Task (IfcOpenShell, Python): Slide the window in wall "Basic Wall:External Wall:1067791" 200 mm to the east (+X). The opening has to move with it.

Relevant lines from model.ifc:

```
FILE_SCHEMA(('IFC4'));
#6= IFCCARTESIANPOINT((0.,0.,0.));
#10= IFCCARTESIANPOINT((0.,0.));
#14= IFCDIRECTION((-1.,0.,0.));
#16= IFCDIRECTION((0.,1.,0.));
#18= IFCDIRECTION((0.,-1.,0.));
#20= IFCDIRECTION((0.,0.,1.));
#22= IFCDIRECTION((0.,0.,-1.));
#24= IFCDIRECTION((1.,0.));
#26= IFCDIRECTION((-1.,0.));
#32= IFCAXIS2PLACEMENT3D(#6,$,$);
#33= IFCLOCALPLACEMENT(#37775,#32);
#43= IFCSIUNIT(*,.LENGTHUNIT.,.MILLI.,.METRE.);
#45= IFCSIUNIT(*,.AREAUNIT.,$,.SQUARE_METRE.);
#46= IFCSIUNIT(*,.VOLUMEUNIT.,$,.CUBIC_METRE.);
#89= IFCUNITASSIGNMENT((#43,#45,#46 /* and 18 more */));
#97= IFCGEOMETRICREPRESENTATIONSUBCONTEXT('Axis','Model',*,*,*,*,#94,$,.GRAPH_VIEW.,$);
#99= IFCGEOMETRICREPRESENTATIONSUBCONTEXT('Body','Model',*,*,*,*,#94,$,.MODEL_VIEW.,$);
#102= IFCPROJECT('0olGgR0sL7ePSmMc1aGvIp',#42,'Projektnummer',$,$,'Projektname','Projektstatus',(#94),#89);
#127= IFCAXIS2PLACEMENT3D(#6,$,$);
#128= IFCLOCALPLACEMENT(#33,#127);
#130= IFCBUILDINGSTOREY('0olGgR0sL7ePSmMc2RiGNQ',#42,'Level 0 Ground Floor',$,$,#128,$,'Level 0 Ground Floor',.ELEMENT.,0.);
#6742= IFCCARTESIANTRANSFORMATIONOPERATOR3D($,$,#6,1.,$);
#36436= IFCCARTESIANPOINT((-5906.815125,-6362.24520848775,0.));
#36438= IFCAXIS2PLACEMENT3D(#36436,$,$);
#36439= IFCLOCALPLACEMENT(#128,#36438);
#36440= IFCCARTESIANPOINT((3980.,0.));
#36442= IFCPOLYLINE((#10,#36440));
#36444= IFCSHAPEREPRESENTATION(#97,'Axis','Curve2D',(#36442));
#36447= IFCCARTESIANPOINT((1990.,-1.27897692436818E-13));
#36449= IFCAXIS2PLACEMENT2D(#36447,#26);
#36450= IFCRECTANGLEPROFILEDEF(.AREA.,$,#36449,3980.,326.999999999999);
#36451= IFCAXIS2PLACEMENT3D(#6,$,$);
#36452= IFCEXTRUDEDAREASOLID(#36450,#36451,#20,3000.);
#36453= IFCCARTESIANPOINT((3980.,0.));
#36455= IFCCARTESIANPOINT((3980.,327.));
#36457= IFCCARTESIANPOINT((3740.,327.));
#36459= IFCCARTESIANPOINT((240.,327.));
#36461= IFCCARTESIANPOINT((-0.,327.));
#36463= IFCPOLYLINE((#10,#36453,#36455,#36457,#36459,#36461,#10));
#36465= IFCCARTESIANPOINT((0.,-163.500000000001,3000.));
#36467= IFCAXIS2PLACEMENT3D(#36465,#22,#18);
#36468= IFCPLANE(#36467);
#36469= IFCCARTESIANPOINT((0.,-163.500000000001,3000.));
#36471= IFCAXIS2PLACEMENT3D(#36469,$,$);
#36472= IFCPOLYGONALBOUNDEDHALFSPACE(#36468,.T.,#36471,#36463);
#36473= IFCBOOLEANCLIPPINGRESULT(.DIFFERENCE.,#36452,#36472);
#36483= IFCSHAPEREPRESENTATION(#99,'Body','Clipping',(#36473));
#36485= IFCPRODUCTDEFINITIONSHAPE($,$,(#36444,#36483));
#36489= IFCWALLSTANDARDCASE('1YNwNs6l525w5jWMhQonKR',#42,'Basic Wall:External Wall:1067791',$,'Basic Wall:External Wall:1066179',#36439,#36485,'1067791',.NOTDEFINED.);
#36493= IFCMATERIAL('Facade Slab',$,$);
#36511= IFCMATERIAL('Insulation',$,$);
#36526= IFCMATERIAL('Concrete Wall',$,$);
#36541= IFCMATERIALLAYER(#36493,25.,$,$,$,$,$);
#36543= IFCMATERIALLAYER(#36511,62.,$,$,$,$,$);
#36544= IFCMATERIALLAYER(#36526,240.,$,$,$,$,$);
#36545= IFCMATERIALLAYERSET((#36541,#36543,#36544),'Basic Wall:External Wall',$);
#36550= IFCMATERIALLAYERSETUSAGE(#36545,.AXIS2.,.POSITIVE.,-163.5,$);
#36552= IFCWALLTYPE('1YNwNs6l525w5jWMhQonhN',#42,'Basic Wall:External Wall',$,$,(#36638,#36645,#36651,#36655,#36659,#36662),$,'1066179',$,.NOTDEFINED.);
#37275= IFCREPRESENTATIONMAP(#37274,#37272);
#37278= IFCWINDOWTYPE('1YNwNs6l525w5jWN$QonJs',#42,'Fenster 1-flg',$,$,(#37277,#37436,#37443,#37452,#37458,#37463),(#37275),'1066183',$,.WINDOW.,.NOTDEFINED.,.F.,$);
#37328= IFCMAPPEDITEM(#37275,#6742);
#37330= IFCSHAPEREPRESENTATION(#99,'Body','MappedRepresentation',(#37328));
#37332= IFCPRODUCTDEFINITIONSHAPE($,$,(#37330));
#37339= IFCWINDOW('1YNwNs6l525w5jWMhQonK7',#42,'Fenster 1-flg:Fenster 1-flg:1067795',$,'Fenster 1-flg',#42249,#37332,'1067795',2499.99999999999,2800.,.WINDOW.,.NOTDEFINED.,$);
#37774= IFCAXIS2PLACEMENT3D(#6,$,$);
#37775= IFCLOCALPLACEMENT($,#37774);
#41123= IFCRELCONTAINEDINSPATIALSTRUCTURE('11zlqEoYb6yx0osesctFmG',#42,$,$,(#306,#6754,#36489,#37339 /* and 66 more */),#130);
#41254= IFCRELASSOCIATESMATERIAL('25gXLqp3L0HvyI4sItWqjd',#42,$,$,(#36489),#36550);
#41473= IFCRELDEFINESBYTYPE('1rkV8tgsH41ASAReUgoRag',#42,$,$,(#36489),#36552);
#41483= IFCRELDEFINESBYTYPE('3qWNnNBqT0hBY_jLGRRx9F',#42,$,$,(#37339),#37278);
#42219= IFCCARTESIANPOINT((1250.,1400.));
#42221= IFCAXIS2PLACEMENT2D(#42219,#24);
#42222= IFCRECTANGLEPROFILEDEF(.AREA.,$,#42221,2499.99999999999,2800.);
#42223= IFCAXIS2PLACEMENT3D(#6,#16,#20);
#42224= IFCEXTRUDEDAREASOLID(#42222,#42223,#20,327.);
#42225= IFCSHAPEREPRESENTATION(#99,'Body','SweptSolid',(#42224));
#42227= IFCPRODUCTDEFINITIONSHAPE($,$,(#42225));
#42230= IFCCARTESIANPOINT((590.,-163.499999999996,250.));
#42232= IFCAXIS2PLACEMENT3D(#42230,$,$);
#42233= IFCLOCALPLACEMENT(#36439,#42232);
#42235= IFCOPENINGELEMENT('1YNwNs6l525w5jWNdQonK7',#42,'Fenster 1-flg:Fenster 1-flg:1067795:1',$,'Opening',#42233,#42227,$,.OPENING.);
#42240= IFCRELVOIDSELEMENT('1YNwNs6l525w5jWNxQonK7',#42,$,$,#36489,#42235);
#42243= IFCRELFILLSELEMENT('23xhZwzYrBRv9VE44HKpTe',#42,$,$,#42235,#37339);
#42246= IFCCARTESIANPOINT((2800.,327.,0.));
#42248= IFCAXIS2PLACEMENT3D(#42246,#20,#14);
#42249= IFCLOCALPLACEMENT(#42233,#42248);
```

```python
import ifcopenshell
import ifcopenshell.api.geometry
import ifcopenshell.util.placement
import ifcopenshell.util.unit

model = ifcopenshell.open("model.ifc")
unit_scale = ifcopenshell.util.unit.calculate_unit_scale(model)

window = model.by_guid("1YNwNs6l525w5jWMhQonK7")
opening = window.FillsVoids[0].RelatingOpeningElement
wall = opening.VoidsElements[0].RelatingBuildingElement

wall_matrix = ifcopenshell.util.placement.get_local_placement(wall.ObjectPlacement)
shift = wall_matrix[:3, 0] * 0.2 / unit_scale
before = ifcopenshell.util.placement.get_local_placement(window.ObjectPlacement)[:3, 3].copy()

# The window is placed relative to its opening, so it follows when the opening moves.
matrix = ifcopenshell.util.placement.get_local_placement(opening.ObjectPlacement)
matrix[:3, 3] += shift
ifcopenshell.api.geometry.edit_object_placement(
    model, product=opening, matrix=matrix, is_si=False, should_transform_children=True
)

after = ifcopenshell.util.placement.get_local_placement(window.ObjectPlacement)[:3, 3]
print("window moved by", (after - before).round(3) + 0.0)

model.write("model_rev.ifc")
```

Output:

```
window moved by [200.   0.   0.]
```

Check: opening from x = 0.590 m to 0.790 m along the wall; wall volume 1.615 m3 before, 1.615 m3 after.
